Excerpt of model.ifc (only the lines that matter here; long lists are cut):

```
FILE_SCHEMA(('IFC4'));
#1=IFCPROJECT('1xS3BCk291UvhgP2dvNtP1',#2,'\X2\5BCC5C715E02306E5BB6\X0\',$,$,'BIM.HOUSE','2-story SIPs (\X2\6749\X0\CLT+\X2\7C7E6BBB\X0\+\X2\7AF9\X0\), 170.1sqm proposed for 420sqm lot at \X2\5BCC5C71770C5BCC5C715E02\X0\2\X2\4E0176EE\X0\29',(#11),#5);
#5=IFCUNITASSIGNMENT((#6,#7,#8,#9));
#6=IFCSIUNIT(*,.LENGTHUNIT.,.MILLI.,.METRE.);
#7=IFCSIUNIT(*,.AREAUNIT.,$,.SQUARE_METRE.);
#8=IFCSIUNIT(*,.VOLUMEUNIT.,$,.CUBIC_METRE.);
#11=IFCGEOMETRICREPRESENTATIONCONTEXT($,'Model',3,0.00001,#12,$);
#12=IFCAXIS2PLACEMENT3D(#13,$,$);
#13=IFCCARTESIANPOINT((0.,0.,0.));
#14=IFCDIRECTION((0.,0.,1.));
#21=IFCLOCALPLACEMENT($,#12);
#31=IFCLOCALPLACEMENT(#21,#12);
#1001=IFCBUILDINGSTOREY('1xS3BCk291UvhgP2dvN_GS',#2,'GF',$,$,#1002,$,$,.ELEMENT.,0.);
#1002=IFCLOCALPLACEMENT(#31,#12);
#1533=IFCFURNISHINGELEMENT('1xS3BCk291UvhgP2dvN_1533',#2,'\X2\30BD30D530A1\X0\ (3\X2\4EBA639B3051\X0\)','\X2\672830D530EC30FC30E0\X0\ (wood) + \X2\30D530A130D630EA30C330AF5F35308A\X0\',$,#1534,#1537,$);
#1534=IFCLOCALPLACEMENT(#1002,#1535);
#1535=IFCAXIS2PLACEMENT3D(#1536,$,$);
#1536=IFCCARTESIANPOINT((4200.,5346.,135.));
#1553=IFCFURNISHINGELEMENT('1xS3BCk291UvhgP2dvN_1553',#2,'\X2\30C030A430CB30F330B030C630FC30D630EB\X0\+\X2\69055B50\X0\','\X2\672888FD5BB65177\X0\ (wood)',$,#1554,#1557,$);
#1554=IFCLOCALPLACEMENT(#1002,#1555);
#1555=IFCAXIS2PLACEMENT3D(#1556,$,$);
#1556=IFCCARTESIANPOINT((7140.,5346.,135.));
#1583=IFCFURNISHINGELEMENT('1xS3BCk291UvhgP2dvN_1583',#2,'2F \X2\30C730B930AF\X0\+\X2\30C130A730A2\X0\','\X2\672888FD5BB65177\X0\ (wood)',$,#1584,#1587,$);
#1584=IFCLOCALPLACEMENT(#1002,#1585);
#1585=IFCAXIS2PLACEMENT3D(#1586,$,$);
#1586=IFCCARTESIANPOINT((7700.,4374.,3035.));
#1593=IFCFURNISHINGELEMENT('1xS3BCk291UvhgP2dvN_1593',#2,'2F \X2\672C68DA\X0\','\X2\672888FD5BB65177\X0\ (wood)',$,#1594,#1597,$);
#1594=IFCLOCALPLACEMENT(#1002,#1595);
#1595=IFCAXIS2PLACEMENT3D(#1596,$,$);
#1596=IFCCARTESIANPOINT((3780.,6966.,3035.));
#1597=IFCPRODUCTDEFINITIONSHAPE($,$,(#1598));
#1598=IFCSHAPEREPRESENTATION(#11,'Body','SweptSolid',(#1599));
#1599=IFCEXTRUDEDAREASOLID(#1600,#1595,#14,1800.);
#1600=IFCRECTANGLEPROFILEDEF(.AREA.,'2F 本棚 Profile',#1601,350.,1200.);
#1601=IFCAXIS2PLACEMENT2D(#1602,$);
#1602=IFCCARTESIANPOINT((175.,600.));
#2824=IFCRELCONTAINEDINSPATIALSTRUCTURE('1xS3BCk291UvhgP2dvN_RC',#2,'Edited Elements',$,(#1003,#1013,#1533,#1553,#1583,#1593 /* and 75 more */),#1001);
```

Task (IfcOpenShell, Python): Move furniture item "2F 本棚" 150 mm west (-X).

```python
import ifcopenshell
import ifcopenshell.api.geometry
import ifcopenshell.util.placement
import ifcopenshell.util.unit

model = ifcopenshell.open("model.ifc")
unit_scale = ifcopenshell.util.unit.calculate_unit_scale(model)

item = model.by_guid("1xS3BCk291UvhgP2dvN_1593")
matrix = ifcopenshell.util.placement.get_local_placement(item.ObjectPlacement)
matrix[0, 3] -= 0.15 / unit_scale
ifcopenshell.api.geometry.edit_object_placement(model, product=item, matrix=matrix, is_si=False)

print(ifcopenshell.util.placement.get_local_placement(item.ObjectPlacement).round(3) + 0.0)

model.write("model_rev.ifc")
```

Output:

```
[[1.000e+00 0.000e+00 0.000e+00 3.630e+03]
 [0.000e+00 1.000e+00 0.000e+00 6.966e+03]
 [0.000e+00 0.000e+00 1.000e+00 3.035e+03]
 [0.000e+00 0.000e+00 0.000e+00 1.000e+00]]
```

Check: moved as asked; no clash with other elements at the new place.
